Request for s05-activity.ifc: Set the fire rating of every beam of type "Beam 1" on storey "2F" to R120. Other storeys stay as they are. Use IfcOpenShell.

First a look at what the model holds.

```python
import ifcopenshell
import ifcopenshell.util.element

model = ifcopenshell.open("s05-activity.ifc")
print(model.schema)
storey = next(s for s in model.by_type("IfcBuildingStorey") if s.Name == "2F")
beams = [e for e in ifcopenshell.util.element.get_decomposition(storey) if e.is_a("IfcBeam")]
seen = {}
for e in beams:
    element_type = ifcopenshell.util.element.get_type(e)
    key = (element_type.Name if element_type != e and element_type else None, ifcopenshell.util.element.get_pset(e, "Pset_BeamCommon", "FireRating"))
    seen[key] = seen.get(key, 0) + 1
for (name, value), count in sorted(seen.items(), key=str):
    print(count, "x", name, "|", value)
```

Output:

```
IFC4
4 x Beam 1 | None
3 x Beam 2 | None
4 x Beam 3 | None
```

```python
import ifcopenshell
import ifcopenshell.api.pset
import ifcopenshell.util.element

model = ifcopenshell.open("s05-activity.ifc")

storey = next(s for s in model.by_type("IfcBuildingStorey") if s.Name == "2F")
beams = [e for e in ifcopenshell.util.element.get_decomposition(storey) if e.is_a("IfcBeam")]

count = 0
for e in beams:
    element_type = ifcopenshell.util.element.get_type(e)
    if element_type in (None, e) or element_type.Name != "Beam 1":
        continue
    # add_pset returns the element's existing set when there is one.
    pset = ifcopenshell.api.pset.add_pset(model, product=e, name="Pset_BeamCommon")
    ifcopenshell.api.pset.edit_pset(model, pset=pset, properties={"FireRating": "R120"})
    count += 1

print(count, "beams updated")

model.write("s05-activity_v2.ifc")
```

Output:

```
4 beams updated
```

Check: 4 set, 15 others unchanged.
